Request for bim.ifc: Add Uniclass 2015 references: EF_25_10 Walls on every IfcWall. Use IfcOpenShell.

First a look at what the model holds.

```python
import ifcopenshell

model = ifcopenshell.open("bim.ifc")
print(model.schema)
print("classifications:", [c.Name for c in model.by_type("IfcClassification")])
for ifc_class in ("IfcDoor", "IfcRoof", "IfcStair", "IfcWall", "IfcWindow"):
    print(ifc_class, len(model.by_type(ifc_class)))
```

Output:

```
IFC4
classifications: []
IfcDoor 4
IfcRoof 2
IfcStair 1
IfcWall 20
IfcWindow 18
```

```python
import ifcopenshell
import ifcopenshell.api.classification

model = ifcopenshell.open("bim.ifc")

system = ifcopenshell.api.classification.add_classification(model, classification="Uniclass 2015")

codes = {
    "IfcWall": ("EF_25_10", "Walls"),
}
for ifc_class, (code, name) in codes.items():
    products = model.by_type(ifc_class)
    ifcopenshell.api.classification.add_reference(
        model, products=products, classification=system, identification=code, name=name
    )
    print(code, len(products))

model.write("bim_edited.ifc")
```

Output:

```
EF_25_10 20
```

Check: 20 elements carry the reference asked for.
